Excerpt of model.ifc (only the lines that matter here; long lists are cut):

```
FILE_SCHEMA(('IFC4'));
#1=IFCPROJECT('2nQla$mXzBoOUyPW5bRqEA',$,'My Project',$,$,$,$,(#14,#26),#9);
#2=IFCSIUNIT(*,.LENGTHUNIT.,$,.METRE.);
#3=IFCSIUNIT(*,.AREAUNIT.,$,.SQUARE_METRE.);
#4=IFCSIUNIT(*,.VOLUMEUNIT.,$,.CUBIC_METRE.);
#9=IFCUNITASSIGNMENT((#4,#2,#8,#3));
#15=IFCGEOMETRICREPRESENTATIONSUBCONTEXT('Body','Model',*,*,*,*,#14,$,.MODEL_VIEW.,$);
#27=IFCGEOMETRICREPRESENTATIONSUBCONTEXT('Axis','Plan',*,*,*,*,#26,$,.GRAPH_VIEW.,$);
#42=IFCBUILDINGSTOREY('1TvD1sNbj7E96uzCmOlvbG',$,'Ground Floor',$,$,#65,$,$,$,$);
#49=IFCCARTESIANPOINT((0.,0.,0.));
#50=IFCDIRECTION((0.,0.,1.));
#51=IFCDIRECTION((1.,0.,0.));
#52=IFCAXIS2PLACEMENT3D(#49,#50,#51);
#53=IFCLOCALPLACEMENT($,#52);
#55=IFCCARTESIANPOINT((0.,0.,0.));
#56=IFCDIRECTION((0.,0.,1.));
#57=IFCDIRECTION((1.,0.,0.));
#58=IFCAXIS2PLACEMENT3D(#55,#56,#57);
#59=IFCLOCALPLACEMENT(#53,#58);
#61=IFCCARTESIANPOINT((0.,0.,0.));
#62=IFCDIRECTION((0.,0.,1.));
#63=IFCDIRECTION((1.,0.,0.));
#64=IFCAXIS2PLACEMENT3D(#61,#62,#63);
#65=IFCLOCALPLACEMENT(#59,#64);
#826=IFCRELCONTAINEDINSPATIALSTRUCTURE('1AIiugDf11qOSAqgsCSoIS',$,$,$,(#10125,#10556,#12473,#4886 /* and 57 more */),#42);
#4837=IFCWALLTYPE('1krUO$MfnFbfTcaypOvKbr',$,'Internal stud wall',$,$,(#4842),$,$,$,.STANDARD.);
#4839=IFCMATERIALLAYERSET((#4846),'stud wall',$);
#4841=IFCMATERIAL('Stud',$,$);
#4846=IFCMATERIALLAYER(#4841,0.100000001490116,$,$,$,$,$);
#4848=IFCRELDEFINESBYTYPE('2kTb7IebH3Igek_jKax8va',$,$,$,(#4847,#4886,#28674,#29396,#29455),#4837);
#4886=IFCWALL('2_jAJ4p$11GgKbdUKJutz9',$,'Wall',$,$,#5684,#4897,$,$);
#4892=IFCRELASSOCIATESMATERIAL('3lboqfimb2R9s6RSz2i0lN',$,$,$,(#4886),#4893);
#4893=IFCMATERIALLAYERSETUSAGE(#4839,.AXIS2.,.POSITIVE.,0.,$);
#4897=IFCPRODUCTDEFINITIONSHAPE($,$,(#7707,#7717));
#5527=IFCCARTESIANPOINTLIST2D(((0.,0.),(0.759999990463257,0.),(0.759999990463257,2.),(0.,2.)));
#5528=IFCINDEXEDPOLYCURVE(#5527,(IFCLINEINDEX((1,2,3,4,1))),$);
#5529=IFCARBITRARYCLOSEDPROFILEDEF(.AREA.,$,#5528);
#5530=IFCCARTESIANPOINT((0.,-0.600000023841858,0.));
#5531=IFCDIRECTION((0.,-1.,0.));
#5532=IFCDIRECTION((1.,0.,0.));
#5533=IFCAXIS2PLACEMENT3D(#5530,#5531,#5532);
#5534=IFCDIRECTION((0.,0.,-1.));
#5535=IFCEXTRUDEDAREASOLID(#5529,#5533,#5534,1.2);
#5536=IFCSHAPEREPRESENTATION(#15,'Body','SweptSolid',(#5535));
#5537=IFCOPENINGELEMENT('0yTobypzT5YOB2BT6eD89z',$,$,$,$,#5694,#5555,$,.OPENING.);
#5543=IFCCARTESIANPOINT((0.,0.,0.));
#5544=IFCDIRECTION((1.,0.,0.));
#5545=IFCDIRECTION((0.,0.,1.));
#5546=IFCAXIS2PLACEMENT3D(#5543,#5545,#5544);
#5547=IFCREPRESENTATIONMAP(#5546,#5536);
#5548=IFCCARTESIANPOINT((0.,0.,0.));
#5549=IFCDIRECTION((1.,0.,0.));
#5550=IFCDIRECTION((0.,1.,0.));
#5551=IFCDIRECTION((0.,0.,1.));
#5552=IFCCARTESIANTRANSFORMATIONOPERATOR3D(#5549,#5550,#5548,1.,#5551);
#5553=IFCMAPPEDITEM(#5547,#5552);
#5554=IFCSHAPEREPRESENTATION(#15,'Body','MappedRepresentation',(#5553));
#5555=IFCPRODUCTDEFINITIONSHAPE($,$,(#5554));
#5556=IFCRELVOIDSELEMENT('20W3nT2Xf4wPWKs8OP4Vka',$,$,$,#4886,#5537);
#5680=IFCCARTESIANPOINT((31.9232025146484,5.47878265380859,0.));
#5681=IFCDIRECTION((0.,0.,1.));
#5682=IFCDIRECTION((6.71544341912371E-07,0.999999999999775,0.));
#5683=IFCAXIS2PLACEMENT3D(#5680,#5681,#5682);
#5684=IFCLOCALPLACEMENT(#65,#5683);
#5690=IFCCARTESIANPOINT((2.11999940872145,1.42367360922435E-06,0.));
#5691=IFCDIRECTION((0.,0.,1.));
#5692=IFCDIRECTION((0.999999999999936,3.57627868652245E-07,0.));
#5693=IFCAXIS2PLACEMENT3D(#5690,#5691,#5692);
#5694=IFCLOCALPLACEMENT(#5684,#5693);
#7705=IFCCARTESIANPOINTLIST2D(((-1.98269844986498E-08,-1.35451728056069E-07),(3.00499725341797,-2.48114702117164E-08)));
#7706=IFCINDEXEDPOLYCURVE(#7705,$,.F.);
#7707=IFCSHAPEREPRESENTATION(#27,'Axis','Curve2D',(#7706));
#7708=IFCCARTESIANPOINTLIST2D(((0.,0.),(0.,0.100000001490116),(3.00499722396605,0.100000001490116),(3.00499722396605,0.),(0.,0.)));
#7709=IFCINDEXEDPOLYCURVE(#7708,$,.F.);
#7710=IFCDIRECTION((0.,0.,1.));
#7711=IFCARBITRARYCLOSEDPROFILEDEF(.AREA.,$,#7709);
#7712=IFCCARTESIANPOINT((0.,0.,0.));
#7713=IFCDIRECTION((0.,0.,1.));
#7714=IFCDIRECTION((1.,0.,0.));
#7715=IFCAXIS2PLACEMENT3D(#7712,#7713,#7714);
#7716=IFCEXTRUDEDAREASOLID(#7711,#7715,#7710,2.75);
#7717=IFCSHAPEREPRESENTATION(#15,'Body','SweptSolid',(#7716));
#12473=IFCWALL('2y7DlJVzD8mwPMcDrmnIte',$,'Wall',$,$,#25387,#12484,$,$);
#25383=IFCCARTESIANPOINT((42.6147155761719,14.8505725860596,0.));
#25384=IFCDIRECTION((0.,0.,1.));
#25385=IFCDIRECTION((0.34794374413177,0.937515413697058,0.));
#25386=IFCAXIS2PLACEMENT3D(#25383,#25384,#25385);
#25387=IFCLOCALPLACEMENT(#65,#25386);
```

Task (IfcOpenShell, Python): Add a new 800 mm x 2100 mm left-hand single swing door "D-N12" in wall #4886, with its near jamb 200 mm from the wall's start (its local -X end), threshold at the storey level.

```python
import numpy as np
import ifcopenshell
import ifcopenshell.api.feature
import ifcopenshell.api.geometry
import ifcopenshell.api.root
import ifcopenshell.api.spatial
import ifcopenshell.geom
import ifcopenshell.util.element
import ifcopenshell.util.placement
import ifcopenshell.util.representation
import ifcopenshell.util.shape
import ifcopenshell.util.unit

model = ifcopenshell.open("model.ifc")
unit_scale = ifcopenshell.util.unit.calculate_unit_scale(model)
settings = ifcopenshell.geom.settings()


def volume(element):
    """Net volume in cubic metres, openings subtracted."""
    shape = ifcopenshell.geom.create_shape(settings, element)
    return ifcopenshell.util.shape.get_volume(shape.geometry)


wall = model.by_guid("2_jAJ4p$11GgKbdUKJutz9")
storey = ifcopenshell.util.element.get_container(wall, ifc_class="IfcBuildingStorey")
context = ifcopenshell.util.representation.get_context(model, "Model", "Body", "MODEL_VIEW")
before = volume(wall)

width, height, from_end, sill = 0.8, 2.1, 0.2, 0.0  # metres

# The wall runs along its own X axis, and the end named is its -X end.
wall_shape = ifcopenshell.geom.create_shape(settings, wall)
x, y, z = ifcopenshell.util.shape.get_vertices(wall_shape.geometry).T
start = x.min() + from_end
face, thickness = float(y.min()), float(y.max() - y.min())
wall_matrix = ifcopenshell.util.placement.get_local_placement(wall.ObjectPlacement)
level = ifcopenshell.util.placement.get_local_placement(storey.ObjectPlacement)[2, 3]


def in_wall(x, y):
    """Placement at x, y metres in the wall's axes, at sill height."""
    matrix = wall_matrix.copy()
    matrix[:, 3] = wall_matrix @ np.array([x / unit_scale, y / unit_scale, 0.0, 1.0])
    matrix[2, 3] = level + sill / unit_scale
    return matrix


# Opening: a box that overshoots both wall faces by 50 mm.
opening = ifcopenshell.api.root.create_entity(model, ifc_class="IfcOpeningElement", predefined_type="OPENING")
box = ifcopenshell.api.geometry.add_wall_representation(
    model, context=context, length=width, height=height, thickness=thickness + 0.1
)
ifcopenshell.api.geometry.assign_representation(model, product=opening, representation=box)
ifcopenshell.api.geometry.edit_object_placement(model, product=opening, matrix=in_wall(start, face - 0.05), is_si=False)
ifcopenshell.api.feature.add_feature(model, feature=opening, element=wall)

door = ifcopenshell.api.root.create_entity(model, ifc_class="IfcDoor", name="D-N12", predefined_type="DOOR")
door.OverallWidth, door.OverallHeight = width / unit_scale, height / unit_scale
door.OperationType = "SINGLE_SWING_LEFT"
body = ifcopenshell.api.geometry.add_door_representation(
    model,
    context=context,
    overall_width=door.OverallWidth,
    overall_height=door.OverallHeight,
    operation_type="SINGLE_SWING_LEFT",
    lining_properties={"LiningDepth": thickness / unit_scale, "ThresholdDepth": thickness / unit_scale},
)
ifcopenshell.api.geometry.assign_representation(model, product=door, representation=body)
ifcopenshell.api.spatial.assign_container(model, products=[door], relating_structure=storey)
ifcopenshell.api.feature.add_filling(model, opening=opening, element=door)

# The lining spans the wall, so the door starts at the wall face.
ifcopenshell.api.geometry.edit_object_placement(model, product=door, matrix=in_wall(start, face), is_si=False)

after = volume(wall)

print(f"wall volume {before:.3f} -> {after:.3f} m3")

model.write("model_updated.ifc")
```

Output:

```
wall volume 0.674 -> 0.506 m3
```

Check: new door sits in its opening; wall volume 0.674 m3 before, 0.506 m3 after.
